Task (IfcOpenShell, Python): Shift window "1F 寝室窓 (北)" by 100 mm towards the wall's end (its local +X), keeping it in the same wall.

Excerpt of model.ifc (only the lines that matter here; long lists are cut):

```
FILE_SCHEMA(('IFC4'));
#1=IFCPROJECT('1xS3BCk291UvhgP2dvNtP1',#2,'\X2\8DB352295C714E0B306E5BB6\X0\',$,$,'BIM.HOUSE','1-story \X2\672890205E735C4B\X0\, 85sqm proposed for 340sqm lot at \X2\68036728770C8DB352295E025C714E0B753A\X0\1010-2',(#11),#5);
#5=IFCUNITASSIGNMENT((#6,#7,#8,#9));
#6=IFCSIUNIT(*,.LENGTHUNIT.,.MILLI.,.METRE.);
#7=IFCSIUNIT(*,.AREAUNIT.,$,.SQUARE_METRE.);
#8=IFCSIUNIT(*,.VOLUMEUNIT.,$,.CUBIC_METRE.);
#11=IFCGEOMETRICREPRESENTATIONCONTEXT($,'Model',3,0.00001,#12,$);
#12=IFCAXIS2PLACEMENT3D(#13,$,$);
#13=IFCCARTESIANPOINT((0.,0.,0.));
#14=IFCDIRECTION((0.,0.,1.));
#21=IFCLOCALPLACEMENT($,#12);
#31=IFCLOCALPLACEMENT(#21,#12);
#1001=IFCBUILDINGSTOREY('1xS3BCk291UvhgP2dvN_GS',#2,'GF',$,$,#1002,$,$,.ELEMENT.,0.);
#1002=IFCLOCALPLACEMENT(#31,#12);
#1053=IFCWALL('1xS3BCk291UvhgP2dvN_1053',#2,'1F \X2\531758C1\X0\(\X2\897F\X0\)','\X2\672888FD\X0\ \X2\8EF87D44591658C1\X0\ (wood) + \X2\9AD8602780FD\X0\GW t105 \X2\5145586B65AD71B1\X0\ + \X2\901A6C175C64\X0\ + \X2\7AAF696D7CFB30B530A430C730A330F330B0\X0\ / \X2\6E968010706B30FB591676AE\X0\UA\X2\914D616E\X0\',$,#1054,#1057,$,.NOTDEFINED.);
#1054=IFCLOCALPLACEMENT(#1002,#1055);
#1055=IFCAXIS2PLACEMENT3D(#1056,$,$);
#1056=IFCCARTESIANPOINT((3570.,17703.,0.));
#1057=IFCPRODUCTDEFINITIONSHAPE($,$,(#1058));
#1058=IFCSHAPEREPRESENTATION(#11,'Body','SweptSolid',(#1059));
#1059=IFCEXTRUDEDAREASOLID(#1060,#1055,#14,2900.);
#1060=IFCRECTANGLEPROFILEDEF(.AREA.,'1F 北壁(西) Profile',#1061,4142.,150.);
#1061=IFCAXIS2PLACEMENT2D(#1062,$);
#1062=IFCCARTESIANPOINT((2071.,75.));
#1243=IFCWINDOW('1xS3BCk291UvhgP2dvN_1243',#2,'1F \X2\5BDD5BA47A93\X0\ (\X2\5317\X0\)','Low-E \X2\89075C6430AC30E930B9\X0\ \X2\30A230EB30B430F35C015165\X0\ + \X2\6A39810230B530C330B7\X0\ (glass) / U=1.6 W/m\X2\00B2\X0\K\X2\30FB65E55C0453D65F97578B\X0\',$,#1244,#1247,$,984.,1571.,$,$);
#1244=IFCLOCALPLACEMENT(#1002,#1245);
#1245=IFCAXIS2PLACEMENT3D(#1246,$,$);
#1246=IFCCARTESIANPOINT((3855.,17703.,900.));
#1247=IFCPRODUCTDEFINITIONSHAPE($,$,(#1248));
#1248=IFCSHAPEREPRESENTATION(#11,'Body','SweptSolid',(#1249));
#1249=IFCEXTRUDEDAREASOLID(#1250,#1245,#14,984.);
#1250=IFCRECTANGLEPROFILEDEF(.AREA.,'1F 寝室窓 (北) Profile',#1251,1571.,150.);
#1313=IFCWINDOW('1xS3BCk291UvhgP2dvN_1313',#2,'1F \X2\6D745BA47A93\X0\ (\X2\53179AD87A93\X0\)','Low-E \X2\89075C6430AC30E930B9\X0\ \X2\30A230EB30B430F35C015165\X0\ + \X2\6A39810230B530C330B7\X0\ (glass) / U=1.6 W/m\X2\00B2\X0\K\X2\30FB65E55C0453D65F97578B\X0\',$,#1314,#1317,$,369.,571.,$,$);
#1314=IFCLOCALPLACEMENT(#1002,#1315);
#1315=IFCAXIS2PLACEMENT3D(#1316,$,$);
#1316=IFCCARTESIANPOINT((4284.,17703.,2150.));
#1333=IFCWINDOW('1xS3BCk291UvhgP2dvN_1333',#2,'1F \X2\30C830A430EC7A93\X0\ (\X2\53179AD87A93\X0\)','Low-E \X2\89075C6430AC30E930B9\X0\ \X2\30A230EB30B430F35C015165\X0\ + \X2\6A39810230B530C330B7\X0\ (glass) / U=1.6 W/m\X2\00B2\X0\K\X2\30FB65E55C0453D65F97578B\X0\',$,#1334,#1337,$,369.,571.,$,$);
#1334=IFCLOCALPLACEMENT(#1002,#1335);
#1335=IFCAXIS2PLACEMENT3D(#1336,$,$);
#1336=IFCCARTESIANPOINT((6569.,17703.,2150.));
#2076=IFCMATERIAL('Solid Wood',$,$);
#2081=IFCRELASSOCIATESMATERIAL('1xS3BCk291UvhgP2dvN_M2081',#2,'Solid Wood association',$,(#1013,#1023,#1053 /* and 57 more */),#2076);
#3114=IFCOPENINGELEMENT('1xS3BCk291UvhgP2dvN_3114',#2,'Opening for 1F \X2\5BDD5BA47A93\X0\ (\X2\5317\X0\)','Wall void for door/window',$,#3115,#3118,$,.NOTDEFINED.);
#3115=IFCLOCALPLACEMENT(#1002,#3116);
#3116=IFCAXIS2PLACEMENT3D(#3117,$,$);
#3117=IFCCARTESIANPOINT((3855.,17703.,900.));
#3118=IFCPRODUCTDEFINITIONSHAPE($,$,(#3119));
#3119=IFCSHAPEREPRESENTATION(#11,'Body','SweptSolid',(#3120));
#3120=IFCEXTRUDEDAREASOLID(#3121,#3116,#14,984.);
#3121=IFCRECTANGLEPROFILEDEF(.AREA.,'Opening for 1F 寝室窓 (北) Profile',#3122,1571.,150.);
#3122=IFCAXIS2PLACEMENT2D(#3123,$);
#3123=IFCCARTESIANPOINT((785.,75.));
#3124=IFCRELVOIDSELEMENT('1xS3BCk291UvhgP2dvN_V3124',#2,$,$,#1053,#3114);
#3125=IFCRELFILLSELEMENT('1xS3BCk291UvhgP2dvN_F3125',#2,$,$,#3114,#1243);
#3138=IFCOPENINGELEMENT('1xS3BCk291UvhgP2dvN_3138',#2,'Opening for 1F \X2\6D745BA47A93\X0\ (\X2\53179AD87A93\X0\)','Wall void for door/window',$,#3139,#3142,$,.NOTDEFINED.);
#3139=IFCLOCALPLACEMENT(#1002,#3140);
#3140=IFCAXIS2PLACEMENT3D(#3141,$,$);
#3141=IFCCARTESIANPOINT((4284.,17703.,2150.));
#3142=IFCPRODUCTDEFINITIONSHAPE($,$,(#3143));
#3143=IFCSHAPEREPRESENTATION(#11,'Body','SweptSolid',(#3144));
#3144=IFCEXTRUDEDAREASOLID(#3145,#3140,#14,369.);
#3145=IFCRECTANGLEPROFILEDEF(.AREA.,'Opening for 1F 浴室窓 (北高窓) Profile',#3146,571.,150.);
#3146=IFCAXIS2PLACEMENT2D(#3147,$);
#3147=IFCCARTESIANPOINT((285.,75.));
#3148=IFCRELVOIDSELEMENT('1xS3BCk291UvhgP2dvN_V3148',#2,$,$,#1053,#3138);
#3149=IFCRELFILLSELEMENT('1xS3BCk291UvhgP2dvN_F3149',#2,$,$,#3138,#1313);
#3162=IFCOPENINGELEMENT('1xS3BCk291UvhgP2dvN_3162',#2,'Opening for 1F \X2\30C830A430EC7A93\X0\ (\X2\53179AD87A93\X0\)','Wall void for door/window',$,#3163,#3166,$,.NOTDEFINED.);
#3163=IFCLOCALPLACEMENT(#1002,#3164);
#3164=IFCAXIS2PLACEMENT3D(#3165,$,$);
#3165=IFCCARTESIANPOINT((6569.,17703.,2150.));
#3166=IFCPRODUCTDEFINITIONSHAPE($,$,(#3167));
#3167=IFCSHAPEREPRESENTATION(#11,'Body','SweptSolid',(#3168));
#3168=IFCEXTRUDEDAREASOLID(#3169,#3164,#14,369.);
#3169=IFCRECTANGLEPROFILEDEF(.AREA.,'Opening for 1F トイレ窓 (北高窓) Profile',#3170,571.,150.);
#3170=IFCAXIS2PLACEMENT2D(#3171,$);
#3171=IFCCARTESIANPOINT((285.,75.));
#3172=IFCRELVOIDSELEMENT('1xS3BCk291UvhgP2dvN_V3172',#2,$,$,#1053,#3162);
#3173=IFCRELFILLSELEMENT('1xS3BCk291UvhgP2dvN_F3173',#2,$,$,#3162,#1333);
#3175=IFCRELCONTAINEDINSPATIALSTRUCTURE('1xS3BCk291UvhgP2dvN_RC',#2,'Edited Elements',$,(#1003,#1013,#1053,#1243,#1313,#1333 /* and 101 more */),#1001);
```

```python
import ifcopenshell
import ifcopenshell.api.geometry
import ifcopenshell.util.placement
import ifcopenshell.util.unit

model = ifcopenshell.open("model.ifc")
unit_scale = ifcopenshell.util.unit.calculate_unit_scale(model)

window = model.by_guid("1xS3BCk291UvhgP2dvN_1243")
opening = window.FillsVoids[0].RelatingOpeningElement
wall = opening.VoidsElements[0].RelatingBuildingElement

wall_matrix = ifcopenshell.util.placement.get_local_placement(wall.ObjectPlacement)
shift = wall_matrix[:3, 0] * 0.1 / unit_scale
before = ifcopenshell.util.placement.get_local_placement(window.ObjectPlacement)[:3, 3].copy()

# The window is not placed relative to its opening, so move both.
for product in (opening, window):
    matrix = ifcopenshell.util.placement.get_local_placement(product.ObjectPlacement)
    matrix[:3, 3] += shift
    ifcopenshell.api.geometry.edit_object_placement(model, product=product, matrix=matrix, is_si=False)

after = ifcopenshell.util.placement.get_local_placement(window.ObjectPlacement)[:3, 3]
print("window moved by", (after - before).round(3) + 0.0)

model.write("model_v2.ifc")
```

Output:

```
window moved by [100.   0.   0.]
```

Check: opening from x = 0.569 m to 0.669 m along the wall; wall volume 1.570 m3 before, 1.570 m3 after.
